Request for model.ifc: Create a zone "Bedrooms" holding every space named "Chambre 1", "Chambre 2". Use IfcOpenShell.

First a look at what the model holds.

```python
import ifcopenshell

model = ifcopenshell.open("model.ifc")
print(model.schema)
seen = {}
for space in model.by_type("IfcSpace"):
    seen[space.LongName] = seen.get(space.LongName, 0) + 1
for name, count in sorted(seen.items(), key=str):
    print(count, "x", name)
print("zones:", [z.Name for z in model.by_type("IfcZone")][:20])
```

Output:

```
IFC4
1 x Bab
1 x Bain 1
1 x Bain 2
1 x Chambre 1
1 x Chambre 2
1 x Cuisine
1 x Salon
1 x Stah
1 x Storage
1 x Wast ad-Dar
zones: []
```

```python
import ifcopenshell
import ifcopenshell.api.group
import ifcopenshell.api.root

model = ifcopenshell.open("model.ifc")

names = {"Chambre 1", "Chambre 2"}
spaces = [s for s in model.by_type("IfcSpace") if s.LongName in names]

zone = ifcopenshell.api.root.create_entity(model, ifc_class="IfcZone", name="Bedrooms")
ifcopenshell.api.group.assign_group(model, products=spaces, group=zone)
print(len(spaces), "spaces in", zone.Name)

model.write("model_rev.ifc")
```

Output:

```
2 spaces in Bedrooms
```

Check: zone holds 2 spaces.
